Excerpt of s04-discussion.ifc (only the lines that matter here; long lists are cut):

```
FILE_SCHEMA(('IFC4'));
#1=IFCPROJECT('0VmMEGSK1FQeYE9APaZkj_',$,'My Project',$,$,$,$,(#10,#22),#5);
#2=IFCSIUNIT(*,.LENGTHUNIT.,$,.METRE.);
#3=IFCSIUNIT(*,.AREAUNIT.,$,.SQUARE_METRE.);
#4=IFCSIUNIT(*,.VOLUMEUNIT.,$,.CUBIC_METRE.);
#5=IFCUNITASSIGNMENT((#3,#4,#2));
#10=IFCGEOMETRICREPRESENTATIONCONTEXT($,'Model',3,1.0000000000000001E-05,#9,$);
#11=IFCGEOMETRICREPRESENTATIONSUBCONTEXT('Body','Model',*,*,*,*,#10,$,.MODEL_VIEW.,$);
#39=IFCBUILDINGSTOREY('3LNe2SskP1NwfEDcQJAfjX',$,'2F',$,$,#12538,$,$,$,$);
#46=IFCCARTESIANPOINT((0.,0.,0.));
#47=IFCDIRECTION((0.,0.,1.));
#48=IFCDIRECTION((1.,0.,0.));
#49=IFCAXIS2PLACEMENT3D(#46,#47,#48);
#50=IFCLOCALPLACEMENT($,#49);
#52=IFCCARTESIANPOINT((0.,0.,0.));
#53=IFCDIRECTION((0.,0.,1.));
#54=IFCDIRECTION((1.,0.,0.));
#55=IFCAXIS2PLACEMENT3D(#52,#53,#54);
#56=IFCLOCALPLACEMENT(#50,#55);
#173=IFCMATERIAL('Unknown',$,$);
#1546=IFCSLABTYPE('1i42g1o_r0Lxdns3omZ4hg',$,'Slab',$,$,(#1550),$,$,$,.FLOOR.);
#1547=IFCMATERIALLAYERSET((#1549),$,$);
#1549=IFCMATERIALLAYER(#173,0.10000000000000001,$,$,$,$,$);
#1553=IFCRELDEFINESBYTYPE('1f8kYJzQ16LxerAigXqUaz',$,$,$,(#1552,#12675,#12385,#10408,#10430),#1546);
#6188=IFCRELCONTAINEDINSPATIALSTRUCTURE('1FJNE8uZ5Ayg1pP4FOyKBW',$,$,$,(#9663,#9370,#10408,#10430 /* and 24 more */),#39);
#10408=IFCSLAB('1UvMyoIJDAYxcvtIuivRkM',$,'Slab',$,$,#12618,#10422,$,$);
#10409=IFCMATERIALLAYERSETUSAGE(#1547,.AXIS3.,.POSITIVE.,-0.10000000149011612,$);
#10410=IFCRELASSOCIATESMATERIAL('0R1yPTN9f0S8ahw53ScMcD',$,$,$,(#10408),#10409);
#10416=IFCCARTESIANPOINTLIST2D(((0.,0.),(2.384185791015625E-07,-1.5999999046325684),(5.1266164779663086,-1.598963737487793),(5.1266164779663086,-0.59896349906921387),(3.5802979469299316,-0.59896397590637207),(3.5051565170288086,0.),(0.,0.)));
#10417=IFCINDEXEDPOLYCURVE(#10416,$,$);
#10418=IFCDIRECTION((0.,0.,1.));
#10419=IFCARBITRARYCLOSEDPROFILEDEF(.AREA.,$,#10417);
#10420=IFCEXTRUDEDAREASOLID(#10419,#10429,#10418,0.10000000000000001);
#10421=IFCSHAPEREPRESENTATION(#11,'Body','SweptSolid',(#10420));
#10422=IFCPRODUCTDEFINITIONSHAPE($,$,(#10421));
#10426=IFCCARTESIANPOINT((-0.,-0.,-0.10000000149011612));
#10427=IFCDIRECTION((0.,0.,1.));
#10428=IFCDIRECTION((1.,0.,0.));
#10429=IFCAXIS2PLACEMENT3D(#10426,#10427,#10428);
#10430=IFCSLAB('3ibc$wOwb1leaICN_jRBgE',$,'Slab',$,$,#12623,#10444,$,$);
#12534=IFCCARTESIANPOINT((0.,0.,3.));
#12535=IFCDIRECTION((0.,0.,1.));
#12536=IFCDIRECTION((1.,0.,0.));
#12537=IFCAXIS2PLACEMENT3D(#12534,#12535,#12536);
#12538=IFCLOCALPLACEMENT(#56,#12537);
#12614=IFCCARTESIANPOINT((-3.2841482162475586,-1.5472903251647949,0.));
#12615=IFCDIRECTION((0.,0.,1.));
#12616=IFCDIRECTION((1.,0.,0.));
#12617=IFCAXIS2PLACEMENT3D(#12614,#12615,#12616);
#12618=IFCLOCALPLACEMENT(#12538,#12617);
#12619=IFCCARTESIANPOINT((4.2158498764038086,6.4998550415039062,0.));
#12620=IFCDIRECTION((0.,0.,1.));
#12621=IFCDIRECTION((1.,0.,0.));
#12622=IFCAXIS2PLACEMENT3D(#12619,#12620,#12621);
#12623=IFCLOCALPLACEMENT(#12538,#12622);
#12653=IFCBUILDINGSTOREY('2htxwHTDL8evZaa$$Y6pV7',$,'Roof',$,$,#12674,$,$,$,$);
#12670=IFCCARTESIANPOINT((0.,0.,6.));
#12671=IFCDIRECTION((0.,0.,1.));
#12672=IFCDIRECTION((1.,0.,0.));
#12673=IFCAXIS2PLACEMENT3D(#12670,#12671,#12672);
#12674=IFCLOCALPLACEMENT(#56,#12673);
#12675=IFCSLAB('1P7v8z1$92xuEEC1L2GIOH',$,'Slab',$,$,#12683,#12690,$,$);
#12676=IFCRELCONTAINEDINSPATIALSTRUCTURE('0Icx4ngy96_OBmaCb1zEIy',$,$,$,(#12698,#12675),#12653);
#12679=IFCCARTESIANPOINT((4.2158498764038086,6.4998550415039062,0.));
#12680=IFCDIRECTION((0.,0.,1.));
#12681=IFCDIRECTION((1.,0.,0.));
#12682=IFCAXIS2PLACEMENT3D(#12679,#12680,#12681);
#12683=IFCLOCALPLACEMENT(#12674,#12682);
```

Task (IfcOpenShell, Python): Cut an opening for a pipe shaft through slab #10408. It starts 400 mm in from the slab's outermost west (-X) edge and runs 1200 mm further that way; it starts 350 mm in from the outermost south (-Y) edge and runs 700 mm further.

```python
import numpy as np
import ifcopenshell
import ifcopenshell.api.feature
import ifcopenshell.api.geometry
import ifcopenshell.api.root
import ifcopenshell.geom
import ifcopenshell.util.placement
import ifcopenshell.util.representation
import ifcopenshell.util.shape
import ifcopenshell.util.unit

model = ifcopenshell.open("s04-discussion.ifc")
unit_scale = ifcopenshell.util.unit.calculate_unit_scale(model)
settings = ifcopenshell.geom.settings()


def volume(element):
    """Net volume in cubic metres, openings subtracted."""
    shape = ifcopenshell.geom.create_shape(settings, element)
    return ifcopenshell.util.shape.get_volume(shape.geometry)


slab = model.by_guid("1UvMyoIJDAYxcvtIuivRkM")
before = volume(slab)

# Extent in the slab's own axes, in metres. The edges named are its -X and -Y sides.
slab_shape = ifcopenshell.geom.create_shape(settings, slab)
vertices = ifcopenshell.util.shape.get_vertices(slab_shape.geometry)
x_min, y_min, bottom = vertices.min(axis=0)
top = vertices[:, 2].max()

opening = ifcopenshell.api.root.create_entity(model, ifc_class="IfcOpeningElement", name="Pipe shaft opening", predefined_type="OPENING")
context = ifcopenshell.util.representation.get_context(model, "Model", "Body", "MODEL_VIEW")
width, depth = 1.2, 0.7
outline = [(0.0, 0.0), (width, 0.0), (width, depth), (0.0, depth), (0.0, 0.0)]
# Overshoot both faces by 50 mm so the cut is clean.
shape = ifcopenshell.api.geometry.add_slab_representation(
    model, context=context, depth=top - bottom + 0.1, polyline=outline
)
ifcopenshell.api.geometry.assign_representation(model, product=opening, representation=shape)

matrix = ifcopenshell.util.placement.get_local_placement(slab.ObjectPlacement)
matrix[:, 3] = matrix @ np.append(np.array([x_min + 0.4, y_min + 0.35, bottom - 0.05]) / unit_scale, 1.0)
ifcopenshell.api.geometry.edit_object_placement(model, product=opening, matrix=matrix, is_si=False)
ifcopenshell.api.feature.add_feature(model, feature=opening, element=slab)

after = volume(slab)

print(f"slab volume {before:.3f} -> {after:.3f} m3")

model.write("s04-discussion_updated.ifc")
```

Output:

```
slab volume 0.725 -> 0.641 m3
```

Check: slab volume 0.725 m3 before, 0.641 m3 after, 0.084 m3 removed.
